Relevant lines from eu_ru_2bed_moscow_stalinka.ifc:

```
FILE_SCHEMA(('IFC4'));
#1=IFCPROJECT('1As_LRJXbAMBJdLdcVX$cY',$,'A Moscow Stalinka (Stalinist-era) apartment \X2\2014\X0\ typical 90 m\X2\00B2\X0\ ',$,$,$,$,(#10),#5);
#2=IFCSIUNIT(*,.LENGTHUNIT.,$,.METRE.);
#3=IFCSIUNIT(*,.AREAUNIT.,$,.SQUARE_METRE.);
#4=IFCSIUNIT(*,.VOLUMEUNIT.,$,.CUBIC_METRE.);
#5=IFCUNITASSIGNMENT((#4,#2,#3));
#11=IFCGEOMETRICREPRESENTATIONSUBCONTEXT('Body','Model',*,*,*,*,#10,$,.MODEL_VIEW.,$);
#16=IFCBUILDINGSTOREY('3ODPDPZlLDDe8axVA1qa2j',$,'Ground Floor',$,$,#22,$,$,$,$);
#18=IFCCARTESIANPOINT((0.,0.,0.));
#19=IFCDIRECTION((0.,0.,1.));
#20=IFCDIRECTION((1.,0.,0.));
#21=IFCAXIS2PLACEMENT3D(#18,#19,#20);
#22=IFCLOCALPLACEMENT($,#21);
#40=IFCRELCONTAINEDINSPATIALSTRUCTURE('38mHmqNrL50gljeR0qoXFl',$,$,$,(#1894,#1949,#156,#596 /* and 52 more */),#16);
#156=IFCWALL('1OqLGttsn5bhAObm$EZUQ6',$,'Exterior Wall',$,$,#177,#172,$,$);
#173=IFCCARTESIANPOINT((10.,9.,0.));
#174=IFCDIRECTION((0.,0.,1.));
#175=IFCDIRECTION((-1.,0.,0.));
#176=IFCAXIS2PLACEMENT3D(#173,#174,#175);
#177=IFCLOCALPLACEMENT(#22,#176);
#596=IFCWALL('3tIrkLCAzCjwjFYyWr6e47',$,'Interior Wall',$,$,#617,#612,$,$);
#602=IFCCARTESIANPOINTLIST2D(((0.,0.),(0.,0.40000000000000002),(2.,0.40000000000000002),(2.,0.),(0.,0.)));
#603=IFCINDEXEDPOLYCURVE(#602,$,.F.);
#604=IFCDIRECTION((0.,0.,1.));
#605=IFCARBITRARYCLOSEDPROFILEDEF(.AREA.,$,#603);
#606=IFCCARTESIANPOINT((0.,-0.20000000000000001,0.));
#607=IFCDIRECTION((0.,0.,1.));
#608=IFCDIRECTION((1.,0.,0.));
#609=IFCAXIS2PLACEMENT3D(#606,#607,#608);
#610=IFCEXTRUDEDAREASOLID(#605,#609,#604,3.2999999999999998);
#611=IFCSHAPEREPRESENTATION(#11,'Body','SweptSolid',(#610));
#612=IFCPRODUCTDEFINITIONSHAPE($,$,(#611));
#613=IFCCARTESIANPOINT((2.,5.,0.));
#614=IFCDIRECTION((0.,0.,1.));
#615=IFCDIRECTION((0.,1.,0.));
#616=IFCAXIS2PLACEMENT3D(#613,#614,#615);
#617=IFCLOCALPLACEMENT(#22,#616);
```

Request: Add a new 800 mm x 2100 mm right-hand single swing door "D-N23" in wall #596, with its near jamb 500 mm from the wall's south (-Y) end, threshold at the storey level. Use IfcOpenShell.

```python
import numpy as np
import ifcopenshell
import ifcopenshell.api.feature
import ifcopenshell.api.geometry
import ifcopenshell.api.root
import ifcopenshell.api.spatial
import ifcopenshell.geom
import ifcopenshell.util.element
import ifcopenshell.util.placement
import ifcopenshell.util.representation
import ifcopenshell.util.shape
import ifcopenshell.util.unit

model = ifcopenshell.open("eu_ru_2bed_moscow_stalinka.ifc")
unit_scale = ifcopenshell.util.unit.calculate_unit_scale(model)
settings = ifcopenshell.geom.settings()


def volume(element):
    """Net volume in cubic metres, openings subtracted."""
    shape = ifcopenshell.geom.create_shape(settings, element)
    return ifcopenshell.util.shape.get_volume(shape.geometry)


wall = model.by_guid("3tIrkLCAzCjwjFYyWr6e47")
storey = ifcopenshell.util.element.get_container(wall, ifc_class="IfcBuildingStorey")
context = ifcopenshell.util.representation.get_context(model, "Model", "Body", "MODEL_VIEW")
before = volume(wall)

width, height, from_end, sill = 0.8, 2.1, 0.5, 0.0  # metres

# The wall runs along its own X axis, and the end named is its -X end.
wall_shape = ifcopenshell.geom.create_shape(settings, wall)
x, y, z = ifcopenshell.util.shape.get_vertices(wall_shape.geometry).T
start = x.min() + from_end
face, thickness = float(y.min()), float(y.max() - y.min())
wall_matrix = ifcopenshell.util.placement.get_local_placement(wall.ObjectPlacement)
level = ifcopenshell.util.placement.get_local_placement(storey.ObjectPlacement)[2, 3]


def in_wall(x, y):
    """Placement at x, y metres in the wall's axes, at sill height."""
    matrix = wall_matrix.copy()
    matrix[:, 3] = wall_matrix @ np.array([x / unit_scale, y / unit_scale, 0.0, 1.0])
    matrix[2, 3] = level + sill / unit_scale
    return matrix


# Opening: a box that overshoots both wall faces by 50 mm.
opening = ifcopenshell.api.root.create_entity(model, ifc_class="IfcOpeningElement", predefined_type="OPENING")
box = ifcopenshell.api.geometry.add_wall_representation(
    model, context=context, length=width, height=height, thickness=thickness + 0.1
)
ifcopenshell.api.geometry.assign_representation(model, product=opening, representation=box)
ifcopenshell.api.geometry.edit_object_placement(model, product=opening, matrix=in_wall(start, face - 0.05), is_si=False)
ifcopenshell.api.feature.add_feature(model, feature=opening, element=wall)

door = ifcopenshell.api.root.create_entity(model, ifc_class="IfcDoor", name="D-N23", predefined_type="DOOR")
door.OverallWidth, door.OverallHeight = width / unit_scale, height / unit_scale
door.OperationType = "SINGLE_SWING_RIGHT"
body = ifcopenshell.api.geometry.add_door_representation(
    model,
    context=context,
    overall_width=door.OverallWidth,
    overall_height=door.OverallHeight,
    operation_type="SINGLE_SWING_RIGHT",
    lining_properties={"LiningDepth": thickness / unit_scale, "ThresholdDepth": thickness / unit_scale},
)
ifcopenshell.api.geometry.assign_representation(model, product=door, representation=body)
ifcopenshell.api.spatial.assign_container(model, products=[door], relating_structure=storey)
ifcopenshell.api.feature.add_filling(model, opening=opening, element=door)

# The lining spans the wall, so the door starts at the wall face.
ifcopenshell.api.geometry.edit_object_placement(model, product=door, matrix=in_wall(start, face), is_si=False)

after = volume(wall)

print(f"wall volume {before:.3f} -> {after:.3f} m3")

model.write("eu_ru_2bed_moscow_stalinka_v2.ifc")
```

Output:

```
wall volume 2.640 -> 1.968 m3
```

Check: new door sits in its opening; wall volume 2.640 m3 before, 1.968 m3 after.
